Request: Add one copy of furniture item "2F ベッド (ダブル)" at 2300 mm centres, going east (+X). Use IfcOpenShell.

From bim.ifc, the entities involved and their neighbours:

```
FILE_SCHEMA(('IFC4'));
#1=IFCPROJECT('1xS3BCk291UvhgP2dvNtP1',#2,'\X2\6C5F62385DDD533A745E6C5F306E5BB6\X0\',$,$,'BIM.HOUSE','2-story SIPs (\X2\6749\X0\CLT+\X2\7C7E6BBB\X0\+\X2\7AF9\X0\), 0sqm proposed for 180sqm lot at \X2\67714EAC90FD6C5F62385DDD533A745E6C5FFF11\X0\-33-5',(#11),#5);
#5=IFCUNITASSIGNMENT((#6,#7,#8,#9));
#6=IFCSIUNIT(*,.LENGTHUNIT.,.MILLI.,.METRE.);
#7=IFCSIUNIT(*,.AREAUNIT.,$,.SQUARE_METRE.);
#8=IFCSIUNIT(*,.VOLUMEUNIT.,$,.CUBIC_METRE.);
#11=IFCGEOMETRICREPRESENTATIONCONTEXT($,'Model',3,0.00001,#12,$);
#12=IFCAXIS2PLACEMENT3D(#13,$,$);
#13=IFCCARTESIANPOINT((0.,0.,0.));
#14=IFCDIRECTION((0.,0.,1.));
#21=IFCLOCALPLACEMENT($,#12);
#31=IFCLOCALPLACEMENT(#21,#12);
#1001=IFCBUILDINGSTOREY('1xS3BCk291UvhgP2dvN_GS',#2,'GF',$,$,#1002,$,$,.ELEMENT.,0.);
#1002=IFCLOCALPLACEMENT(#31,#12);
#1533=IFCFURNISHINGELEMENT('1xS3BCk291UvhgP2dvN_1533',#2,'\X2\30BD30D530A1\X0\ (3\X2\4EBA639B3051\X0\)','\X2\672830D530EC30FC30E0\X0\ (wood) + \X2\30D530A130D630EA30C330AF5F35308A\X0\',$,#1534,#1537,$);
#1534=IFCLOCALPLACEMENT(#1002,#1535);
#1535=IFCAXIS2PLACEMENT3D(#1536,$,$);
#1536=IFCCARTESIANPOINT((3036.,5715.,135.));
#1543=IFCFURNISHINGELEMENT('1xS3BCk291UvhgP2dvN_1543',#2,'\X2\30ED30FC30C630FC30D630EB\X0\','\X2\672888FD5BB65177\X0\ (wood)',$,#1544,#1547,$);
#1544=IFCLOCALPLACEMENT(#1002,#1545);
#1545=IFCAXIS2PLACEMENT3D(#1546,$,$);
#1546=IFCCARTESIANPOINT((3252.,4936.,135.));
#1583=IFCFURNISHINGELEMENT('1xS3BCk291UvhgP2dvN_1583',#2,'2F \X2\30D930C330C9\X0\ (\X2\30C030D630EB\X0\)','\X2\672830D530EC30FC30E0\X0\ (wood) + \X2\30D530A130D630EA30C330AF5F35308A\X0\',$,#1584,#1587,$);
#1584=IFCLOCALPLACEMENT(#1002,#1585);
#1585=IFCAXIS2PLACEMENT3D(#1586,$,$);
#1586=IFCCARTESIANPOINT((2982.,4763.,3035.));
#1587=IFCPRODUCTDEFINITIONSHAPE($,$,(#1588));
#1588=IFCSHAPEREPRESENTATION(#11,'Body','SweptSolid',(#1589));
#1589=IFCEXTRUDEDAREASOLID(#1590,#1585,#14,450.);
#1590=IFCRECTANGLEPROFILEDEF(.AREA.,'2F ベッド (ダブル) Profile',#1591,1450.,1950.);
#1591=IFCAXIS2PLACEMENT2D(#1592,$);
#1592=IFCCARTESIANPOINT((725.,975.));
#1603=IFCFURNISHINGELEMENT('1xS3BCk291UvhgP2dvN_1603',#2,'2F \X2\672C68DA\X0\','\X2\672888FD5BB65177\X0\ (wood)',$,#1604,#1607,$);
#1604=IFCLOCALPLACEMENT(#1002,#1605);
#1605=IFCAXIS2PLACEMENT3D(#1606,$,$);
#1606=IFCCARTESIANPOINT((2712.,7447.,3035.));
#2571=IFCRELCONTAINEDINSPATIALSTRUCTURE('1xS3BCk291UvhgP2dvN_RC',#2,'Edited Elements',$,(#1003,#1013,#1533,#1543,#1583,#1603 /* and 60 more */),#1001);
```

```python
import numpy as np
import ifcopenshell
import ifcopenshell.api.geometry
import ifcopenshell.api.root
import ifcopenshell.util.element
import ifcopenshell.util.placement

model = ifcopenshell.open("bim.ifc")


def reuse_history(source, copy):
    """copy_class also copies each property set's owner history, people and application; keep the originals."""
    for rel in copy.IsDefinedBy:
        if rel.is_a("IfcRelDefinesByProperties") and (history := rel.RelatingPropertyDefinition.OwnerHistory):
            rel.RelatingPropertyDefinition.OwnerHistory = source.OwnerHistory
            ifcopenshell.util.element.remove_deep2(model, history)


source = model.by_guid("1xS3BCk291UvhgP2dvN_1583")
base = ifcopenshell.util.placement.get_local_placement(source.ObjectPlacement)
step = np.array([1.0, 0.0, 0.0]) * 2300.0

for i in range(1, 2):
    copy = ifcopenshell.api.root.copy_class(model, product=source)
    copy.Representation = ifcopenshell.util.element.copy_deep(
        model, source.Representation, exclude=["IfcGeometricRepresentationContext", "IfcRepresentationMap"]
    )
    reuse_history(source, copy)
    matrix = base.copy()
    matrix[:3, 3] += i * step
    print("added at", matrix[:3, 3].round(3) + 0.0)
    ifcopenshell.api.geometry.edit_object_placement(model, product=copy, matrix=matrix, is_si=False)

model.write("bim_edited.ifc")
```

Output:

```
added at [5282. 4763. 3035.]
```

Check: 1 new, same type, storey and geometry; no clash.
